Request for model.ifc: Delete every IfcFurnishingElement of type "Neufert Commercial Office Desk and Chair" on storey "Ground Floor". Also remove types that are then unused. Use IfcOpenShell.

First a look at what the model holds.

```python
import ifcopenshell
import ifcopenshell.util.element

model = ifcopenshell.open("model.ifc")
print(model.schema)
storey = next(s for s in model.by_type("IfcBuildingStorey") if s.Name == "Ground Floor")
furniture = [e for e in ifcopenshell.util.element.get_decomposition(storey) if e.is_a("IfcFurnishingElement")]
seen = {}
for e in furniture:
    element_type = ifcopenshell.util.element.get_type(e)
    name = element_type.Name if element_type not in (None, e) else None
    seen[name] = seen.get(name, 0) + 1
for name, count in sorted(seen.items(), key=str):
    print(count, "x", name)
```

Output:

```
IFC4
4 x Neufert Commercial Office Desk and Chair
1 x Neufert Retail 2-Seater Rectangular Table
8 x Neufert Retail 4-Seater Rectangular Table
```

```python
import ifcopenshell
import ifcopenshell.api.root
import ifcopenshell.util.element

model = ifcopenshell.open("model.ifc")

storey = next(s for s in model.by_type("IfcBuildingStorey") if s.Name == "Ground Floor")
furniture = [e for e in ifcopenshell.util.element.get_decomposition(storey) if e.is_a("IfcFurnishingElement")]
targets = [e for e in furniture if (t := ifcopenshell.util.element.get_type(e)) not in (None, e) and t.Name == "Neufert Commercial Office Desk and Chair"]
types = {ifcopenshell.util.element.get_type(e) for e in targets} - {None, *targets}

for e in targets:
    ifcopenshell.api.root.remove_product(model, product=e)
print(len(targets), "removed")

unused = [t for t in types if not ifcopenshell.util.element.get_types(t)]
for t in unused:
    ifcopenshell.api.root.remove_product(model, product=t)
print(len(unused), "unused types removed")

model.write("model_edited.ifc")
```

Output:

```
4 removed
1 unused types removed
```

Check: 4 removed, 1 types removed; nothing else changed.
